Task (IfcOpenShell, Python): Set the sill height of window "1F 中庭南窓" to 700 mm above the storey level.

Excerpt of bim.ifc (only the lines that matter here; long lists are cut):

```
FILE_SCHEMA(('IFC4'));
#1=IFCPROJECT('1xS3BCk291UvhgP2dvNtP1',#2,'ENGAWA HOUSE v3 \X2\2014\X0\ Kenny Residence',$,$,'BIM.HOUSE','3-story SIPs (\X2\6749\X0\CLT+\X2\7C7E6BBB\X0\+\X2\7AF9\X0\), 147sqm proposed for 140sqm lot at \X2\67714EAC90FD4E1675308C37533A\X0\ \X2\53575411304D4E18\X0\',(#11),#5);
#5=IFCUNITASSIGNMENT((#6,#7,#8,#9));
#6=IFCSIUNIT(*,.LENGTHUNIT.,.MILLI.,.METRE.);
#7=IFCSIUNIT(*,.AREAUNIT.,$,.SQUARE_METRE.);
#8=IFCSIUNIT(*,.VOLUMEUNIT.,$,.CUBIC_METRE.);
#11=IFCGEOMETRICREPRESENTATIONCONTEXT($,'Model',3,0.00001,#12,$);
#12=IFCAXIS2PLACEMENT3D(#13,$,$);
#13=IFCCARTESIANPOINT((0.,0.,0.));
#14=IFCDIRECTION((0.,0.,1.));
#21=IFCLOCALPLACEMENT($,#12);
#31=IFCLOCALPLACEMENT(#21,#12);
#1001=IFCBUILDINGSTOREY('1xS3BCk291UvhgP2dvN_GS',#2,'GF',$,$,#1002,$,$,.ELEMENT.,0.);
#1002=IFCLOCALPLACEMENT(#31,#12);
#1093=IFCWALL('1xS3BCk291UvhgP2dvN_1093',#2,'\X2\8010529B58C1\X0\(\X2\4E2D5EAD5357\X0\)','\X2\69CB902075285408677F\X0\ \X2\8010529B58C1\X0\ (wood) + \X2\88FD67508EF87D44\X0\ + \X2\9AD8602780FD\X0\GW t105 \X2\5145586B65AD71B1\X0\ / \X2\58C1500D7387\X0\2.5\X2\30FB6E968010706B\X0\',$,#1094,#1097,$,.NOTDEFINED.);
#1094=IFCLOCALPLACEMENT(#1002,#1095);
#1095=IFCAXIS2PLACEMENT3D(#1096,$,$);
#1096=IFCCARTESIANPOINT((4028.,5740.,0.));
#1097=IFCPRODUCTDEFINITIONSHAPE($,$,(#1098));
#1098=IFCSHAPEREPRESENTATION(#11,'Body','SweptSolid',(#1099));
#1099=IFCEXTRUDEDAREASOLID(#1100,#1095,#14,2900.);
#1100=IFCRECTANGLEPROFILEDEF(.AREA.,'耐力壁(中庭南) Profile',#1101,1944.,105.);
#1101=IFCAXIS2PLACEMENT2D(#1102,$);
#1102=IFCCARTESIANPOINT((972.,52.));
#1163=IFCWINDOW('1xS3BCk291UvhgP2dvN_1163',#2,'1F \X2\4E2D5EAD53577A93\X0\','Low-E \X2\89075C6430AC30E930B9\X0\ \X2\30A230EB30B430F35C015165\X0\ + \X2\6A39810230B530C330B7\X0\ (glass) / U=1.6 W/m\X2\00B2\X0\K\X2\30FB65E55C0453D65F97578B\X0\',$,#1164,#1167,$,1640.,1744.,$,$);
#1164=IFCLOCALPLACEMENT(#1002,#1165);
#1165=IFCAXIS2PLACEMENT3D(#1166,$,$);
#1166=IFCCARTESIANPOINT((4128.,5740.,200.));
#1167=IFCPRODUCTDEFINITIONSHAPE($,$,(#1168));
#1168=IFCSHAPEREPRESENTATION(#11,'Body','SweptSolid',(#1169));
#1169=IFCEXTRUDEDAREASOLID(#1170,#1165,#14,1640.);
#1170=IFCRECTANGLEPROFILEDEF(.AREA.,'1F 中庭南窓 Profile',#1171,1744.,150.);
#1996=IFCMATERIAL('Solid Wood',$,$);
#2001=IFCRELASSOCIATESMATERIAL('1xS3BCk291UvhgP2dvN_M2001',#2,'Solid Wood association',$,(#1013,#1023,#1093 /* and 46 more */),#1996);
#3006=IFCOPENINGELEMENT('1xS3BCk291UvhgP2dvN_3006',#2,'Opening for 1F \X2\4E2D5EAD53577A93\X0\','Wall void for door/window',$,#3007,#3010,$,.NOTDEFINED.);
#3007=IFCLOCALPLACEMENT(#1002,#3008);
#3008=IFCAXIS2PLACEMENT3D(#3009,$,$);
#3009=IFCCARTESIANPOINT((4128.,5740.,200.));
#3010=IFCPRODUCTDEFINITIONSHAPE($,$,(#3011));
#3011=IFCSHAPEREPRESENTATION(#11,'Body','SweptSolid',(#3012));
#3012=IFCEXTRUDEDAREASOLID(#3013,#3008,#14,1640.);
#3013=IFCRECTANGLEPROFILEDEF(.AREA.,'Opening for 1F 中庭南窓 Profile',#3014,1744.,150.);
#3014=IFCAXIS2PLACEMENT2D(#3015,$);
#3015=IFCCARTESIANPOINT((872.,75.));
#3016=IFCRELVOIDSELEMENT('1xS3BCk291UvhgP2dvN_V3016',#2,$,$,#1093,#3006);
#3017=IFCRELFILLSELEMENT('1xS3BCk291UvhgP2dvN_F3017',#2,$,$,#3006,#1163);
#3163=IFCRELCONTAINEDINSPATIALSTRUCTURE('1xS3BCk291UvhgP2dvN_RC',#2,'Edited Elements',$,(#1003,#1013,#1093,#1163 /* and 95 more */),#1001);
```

```python
import numpy as np
import ifcopenshell
import ifcopenshell.api.geometry
import ifcopenshell.geom
import ifcopenshell.util.element
import ifcopenshell.util.placement
import ifcopenshell.util.shape
import ifcopenshell.util.unit

model = ifcopenshell.open("bim.ifc")
unit_scale = ifcopenshell.util.unit.calculate_unit_scale(model)

window = model.by_id(1163)
opening = window.FillsVoids[0].RelatingOpeningElement
storey = ifcopenshell.util.element.get_container(window, ifc_class="IfcBuildingStorey")
level = ifcopenshell.util.placement.get_local_placement(storey.ObjectPlacement)[2, 3]

# The opening's origin need not be at the sill, so measure its lowest point.
shape = ifcopenshell.geom.create_shape(ifcopenshell.geom.settings(), opening)
bottom = ifcopenshell.util.shape.get_shape_bottom_elevation(shape, shape.geometry) / unit_scale
dz = level + 700.0 - bottom

shift = np.array([0.0, 0.0, dz])
# The window is not placed relative to its opening, so move both.
for product in (opening, window):
    matrix = ifcopenshell.util.placement.get_local_placement(product.ObjectPlacement)
    matrix[:3, 3] += shift
    ifcopenshell.api.geometry.edit_object_placement(model, product=product, matrix=matrix, is_si=False)

print(f"moved by {dz * unit_scale:+.3f} m")

model.write("bim_edited.ifc")
```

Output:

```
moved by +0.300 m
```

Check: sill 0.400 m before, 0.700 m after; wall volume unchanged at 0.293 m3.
